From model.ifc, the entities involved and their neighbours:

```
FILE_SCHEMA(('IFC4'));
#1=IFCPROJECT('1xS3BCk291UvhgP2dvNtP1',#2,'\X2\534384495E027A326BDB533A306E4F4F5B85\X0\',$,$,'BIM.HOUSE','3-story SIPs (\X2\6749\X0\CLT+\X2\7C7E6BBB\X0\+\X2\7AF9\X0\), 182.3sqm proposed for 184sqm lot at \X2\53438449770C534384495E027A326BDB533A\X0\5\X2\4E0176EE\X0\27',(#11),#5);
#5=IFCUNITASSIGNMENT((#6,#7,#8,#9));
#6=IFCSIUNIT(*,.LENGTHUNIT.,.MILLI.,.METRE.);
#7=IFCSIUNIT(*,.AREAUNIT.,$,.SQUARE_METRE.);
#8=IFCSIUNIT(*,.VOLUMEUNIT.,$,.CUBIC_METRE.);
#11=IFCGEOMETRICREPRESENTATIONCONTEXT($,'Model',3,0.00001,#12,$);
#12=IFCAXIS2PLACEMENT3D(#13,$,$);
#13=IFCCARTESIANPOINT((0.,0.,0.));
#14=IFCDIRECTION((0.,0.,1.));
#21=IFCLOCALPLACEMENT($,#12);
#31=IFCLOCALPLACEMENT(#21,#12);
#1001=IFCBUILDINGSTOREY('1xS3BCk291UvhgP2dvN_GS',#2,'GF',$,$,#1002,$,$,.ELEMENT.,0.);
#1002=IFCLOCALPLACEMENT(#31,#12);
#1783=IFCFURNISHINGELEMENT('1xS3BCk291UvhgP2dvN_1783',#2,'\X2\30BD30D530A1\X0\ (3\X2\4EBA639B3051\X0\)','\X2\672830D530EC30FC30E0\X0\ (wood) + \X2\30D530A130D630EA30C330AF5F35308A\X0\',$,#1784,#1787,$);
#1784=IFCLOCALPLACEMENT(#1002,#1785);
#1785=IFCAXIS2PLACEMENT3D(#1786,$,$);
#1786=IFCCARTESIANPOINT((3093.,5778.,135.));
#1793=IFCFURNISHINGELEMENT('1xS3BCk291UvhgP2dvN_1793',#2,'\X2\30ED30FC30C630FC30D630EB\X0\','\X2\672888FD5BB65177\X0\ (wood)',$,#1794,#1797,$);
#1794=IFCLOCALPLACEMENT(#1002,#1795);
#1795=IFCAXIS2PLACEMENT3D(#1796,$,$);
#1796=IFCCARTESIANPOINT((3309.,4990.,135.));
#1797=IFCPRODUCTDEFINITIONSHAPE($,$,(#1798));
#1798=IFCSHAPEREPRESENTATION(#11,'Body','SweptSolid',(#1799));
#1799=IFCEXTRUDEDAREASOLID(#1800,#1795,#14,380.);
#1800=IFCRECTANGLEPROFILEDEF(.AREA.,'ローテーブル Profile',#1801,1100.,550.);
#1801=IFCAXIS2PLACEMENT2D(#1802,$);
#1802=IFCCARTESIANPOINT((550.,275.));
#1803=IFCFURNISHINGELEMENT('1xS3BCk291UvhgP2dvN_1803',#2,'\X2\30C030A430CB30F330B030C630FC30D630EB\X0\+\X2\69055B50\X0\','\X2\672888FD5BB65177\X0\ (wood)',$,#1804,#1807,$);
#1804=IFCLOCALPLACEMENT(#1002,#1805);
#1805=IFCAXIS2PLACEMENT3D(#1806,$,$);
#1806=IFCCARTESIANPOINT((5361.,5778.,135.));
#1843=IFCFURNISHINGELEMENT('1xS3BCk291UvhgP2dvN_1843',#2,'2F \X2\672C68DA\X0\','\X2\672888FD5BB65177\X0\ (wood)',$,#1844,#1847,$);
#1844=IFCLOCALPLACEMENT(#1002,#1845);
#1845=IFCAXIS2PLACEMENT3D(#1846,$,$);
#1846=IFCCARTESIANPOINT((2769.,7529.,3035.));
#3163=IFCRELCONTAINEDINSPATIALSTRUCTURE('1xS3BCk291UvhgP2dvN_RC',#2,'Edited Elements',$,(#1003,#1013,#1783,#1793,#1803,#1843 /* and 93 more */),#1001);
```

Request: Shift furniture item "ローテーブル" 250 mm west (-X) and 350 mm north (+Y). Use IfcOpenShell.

```python
import ifcopenshell
import ifcopenshell.api.geometry
import ifcopenshell.util.placement

model = ifcopenshell.open("model.ifc")

item = model.by_id(1793)
matrix = ifcopenshell.util.placement.get_local_placement(item.ObjectPlacement)
matrix[0, 3] -= 250.0
matrix[1, 3] += 350.0
ifcopenshell.api.geometry.edit_object_placement(model, product=item, matrix=matrix, is_si=False)

print(ifcopenshell.util.placement.get_local_placement(item.ObjectPlacement).round(3) + 0.0)

model.write("model_edited.ifc")
```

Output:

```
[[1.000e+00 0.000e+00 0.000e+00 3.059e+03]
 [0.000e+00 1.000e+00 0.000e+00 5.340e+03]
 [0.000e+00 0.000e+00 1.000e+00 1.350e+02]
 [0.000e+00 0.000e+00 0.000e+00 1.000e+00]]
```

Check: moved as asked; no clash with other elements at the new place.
